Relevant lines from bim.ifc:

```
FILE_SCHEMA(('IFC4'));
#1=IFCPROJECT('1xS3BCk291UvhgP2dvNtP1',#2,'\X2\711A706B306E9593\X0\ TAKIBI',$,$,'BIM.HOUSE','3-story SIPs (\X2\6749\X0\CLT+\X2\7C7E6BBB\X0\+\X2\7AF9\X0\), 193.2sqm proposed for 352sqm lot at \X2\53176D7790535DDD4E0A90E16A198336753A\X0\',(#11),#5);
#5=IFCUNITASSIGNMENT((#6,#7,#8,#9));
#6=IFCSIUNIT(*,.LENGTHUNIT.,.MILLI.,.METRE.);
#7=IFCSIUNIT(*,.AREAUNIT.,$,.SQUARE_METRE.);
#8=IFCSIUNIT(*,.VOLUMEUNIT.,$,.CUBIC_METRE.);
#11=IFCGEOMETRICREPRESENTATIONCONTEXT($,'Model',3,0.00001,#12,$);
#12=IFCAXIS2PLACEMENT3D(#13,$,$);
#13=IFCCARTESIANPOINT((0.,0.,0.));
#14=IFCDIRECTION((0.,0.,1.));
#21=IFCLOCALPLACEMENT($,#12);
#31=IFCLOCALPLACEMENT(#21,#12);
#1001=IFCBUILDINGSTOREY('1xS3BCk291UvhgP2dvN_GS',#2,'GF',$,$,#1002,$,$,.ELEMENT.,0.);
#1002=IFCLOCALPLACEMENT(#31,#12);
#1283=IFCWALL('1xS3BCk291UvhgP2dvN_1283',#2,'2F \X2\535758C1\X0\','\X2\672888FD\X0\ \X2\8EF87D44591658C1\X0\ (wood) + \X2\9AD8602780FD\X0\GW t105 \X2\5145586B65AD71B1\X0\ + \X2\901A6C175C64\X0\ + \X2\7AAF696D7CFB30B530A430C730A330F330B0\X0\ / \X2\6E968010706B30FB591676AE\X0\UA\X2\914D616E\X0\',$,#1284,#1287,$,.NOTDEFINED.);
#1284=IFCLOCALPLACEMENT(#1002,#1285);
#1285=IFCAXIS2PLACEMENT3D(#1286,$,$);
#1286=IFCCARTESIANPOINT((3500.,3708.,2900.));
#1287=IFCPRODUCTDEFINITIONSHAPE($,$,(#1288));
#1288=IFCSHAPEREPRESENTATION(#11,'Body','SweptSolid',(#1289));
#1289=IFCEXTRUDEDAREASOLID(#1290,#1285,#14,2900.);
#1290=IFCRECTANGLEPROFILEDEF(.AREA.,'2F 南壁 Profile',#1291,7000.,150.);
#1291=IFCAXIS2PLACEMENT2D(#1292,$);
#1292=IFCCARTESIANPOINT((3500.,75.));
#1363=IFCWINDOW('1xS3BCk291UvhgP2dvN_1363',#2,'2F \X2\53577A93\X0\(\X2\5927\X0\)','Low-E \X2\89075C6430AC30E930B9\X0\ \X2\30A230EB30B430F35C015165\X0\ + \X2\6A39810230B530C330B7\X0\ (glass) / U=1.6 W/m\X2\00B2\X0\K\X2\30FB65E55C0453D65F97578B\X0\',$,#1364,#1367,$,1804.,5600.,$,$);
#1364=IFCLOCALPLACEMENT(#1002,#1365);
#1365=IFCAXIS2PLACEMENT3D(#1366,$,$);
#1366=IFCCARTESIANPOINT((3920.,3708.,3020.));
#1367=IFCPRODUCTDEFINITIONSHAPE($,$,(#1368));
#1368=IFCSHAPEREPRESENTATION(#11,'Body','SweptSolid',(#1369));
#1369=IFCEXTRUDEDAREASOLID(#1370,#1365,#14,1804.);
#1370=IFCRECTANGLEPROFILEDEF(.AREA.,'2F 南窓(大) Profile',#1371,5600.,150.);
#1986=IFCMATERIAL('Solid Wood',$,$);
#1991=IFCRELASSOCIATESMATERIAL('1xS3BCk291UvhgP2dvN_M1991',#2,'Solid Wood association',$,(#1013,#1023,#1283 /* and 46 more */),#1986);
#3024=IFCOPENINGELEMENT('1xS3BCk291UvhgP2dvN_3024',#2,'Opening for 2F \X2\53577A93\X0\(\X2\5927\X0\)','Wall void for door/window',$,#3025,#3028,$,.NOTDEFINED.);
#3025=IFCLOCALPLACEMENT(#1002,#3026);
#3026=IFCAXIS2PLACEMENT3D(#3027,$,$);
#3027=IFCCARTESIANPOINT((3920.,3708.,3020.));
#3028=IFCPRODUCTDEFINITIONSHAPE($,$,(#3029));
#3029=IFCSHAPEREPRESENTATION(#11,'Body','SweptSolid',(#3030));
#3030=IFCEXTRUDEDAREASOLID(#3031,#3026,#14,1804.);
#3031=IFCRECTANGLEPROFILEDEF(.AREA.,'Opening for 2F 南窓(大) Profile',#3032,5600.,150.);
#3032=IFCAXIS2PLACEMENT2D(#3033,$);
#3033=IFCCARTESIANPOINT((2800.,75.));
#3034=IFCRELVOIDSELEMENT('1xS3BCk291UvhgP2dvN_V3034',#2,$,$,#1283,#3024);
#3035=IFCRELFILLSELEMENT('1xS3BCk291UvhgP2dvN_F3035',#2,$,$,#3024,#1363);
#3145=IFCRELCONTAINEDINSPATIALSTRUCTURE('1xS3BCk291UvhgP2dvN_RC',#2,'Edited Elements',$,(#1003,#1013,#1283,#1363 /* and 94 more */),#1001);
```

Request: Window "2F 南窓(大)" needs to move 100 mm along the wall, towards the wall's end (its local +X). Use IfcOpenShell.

```python
import ifcopenshell
import ifcopenshell.api.geometry
import ifcopenshell.util.placement
import ifcopenshell.util.unit

model = ifcopenshell.open("bim.ifc")
unit_scale = ifcopenshell.util.unit.calculate_unit_scale(model)

window = model.by_guid("1xS3BCk291UvhgP2dvN_1363")
opening = window.FillsVoids[0].RelatingOpeningElement
wall = opening.VoidsElements[0].RelatingBuildingElement

wall_matrix = ifcopenshell.util.placement.get_local_placement(wall.ObjectPlacement)
shift = wall_matrix[:3, 0] * 0.1 / unit_scale
before = ifcopenshell.util.placement.get_local_placement(window.ObjectPlacement)[:3, 3].copy()

# The window is not placed relative to its opening, so move both.
for product in (opening, window):
    matrix = ifcopenshell.util.placement.get_local_placement(product.ObjectPlacement)
    matrix[:3, 3] += shift
    ifcopenshell.api.geometry.edit_object_placement(model, product=product, matrix=matrix, is_si=False)

after = ifcopenshell.util.placement.get_local_placement(window.ObjectPlacement)[:3, 3]
print("window moved by", (after - before).round(3) + 0.0)

model.write("bim-out.ifc")
```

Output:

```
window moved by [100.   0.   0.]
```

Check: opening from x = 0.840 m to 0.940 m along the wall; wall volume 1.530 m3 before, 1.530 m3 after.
